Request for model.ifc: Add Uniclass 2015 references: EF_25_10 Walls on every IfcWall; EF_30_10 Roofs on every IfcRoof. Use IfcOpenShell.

First a look at what the model holds.

```python
import ifcopenshell

model = ifcopenshell.open("model.ifc")
print(model.schema)
print("classifications:", [c.Name for c in model.by_type("IfcClassification")])
for ifc_class in ("IfcDoor", "IfcRoof", "IfcStair", "IfcWall", "IfcWindow"):
    print(ifc_class, len(model.by_type(ifc_class)))
```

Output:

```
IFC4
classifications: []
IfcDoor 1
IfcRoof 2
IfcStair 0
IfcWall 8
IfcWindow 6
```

```python
import ifcopenshell
import ifcopenshell.api.classification

model = ifcopenshell.open("model.ifc")

system = ifcopenshell.api.classification.add_classification(model, classification="Uniclass 2015")

codes = {
    "IfcWall": ("EF_25_10", "Walls"),
    "IfcRoof": ("EF_30_10", "Roofs"),
}
for ifc_class, (code, name) in codes.items():
    products = model.by_type(ifc_class)
    ifcopenshell.api.classification.add_reference(
        model, products=products, classification=system, identification=code, name=name
    )
    print(code, len(products))

model.write("model_updated.ifc")
```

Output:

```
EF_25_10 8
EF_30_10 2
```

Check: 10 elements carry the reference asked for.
